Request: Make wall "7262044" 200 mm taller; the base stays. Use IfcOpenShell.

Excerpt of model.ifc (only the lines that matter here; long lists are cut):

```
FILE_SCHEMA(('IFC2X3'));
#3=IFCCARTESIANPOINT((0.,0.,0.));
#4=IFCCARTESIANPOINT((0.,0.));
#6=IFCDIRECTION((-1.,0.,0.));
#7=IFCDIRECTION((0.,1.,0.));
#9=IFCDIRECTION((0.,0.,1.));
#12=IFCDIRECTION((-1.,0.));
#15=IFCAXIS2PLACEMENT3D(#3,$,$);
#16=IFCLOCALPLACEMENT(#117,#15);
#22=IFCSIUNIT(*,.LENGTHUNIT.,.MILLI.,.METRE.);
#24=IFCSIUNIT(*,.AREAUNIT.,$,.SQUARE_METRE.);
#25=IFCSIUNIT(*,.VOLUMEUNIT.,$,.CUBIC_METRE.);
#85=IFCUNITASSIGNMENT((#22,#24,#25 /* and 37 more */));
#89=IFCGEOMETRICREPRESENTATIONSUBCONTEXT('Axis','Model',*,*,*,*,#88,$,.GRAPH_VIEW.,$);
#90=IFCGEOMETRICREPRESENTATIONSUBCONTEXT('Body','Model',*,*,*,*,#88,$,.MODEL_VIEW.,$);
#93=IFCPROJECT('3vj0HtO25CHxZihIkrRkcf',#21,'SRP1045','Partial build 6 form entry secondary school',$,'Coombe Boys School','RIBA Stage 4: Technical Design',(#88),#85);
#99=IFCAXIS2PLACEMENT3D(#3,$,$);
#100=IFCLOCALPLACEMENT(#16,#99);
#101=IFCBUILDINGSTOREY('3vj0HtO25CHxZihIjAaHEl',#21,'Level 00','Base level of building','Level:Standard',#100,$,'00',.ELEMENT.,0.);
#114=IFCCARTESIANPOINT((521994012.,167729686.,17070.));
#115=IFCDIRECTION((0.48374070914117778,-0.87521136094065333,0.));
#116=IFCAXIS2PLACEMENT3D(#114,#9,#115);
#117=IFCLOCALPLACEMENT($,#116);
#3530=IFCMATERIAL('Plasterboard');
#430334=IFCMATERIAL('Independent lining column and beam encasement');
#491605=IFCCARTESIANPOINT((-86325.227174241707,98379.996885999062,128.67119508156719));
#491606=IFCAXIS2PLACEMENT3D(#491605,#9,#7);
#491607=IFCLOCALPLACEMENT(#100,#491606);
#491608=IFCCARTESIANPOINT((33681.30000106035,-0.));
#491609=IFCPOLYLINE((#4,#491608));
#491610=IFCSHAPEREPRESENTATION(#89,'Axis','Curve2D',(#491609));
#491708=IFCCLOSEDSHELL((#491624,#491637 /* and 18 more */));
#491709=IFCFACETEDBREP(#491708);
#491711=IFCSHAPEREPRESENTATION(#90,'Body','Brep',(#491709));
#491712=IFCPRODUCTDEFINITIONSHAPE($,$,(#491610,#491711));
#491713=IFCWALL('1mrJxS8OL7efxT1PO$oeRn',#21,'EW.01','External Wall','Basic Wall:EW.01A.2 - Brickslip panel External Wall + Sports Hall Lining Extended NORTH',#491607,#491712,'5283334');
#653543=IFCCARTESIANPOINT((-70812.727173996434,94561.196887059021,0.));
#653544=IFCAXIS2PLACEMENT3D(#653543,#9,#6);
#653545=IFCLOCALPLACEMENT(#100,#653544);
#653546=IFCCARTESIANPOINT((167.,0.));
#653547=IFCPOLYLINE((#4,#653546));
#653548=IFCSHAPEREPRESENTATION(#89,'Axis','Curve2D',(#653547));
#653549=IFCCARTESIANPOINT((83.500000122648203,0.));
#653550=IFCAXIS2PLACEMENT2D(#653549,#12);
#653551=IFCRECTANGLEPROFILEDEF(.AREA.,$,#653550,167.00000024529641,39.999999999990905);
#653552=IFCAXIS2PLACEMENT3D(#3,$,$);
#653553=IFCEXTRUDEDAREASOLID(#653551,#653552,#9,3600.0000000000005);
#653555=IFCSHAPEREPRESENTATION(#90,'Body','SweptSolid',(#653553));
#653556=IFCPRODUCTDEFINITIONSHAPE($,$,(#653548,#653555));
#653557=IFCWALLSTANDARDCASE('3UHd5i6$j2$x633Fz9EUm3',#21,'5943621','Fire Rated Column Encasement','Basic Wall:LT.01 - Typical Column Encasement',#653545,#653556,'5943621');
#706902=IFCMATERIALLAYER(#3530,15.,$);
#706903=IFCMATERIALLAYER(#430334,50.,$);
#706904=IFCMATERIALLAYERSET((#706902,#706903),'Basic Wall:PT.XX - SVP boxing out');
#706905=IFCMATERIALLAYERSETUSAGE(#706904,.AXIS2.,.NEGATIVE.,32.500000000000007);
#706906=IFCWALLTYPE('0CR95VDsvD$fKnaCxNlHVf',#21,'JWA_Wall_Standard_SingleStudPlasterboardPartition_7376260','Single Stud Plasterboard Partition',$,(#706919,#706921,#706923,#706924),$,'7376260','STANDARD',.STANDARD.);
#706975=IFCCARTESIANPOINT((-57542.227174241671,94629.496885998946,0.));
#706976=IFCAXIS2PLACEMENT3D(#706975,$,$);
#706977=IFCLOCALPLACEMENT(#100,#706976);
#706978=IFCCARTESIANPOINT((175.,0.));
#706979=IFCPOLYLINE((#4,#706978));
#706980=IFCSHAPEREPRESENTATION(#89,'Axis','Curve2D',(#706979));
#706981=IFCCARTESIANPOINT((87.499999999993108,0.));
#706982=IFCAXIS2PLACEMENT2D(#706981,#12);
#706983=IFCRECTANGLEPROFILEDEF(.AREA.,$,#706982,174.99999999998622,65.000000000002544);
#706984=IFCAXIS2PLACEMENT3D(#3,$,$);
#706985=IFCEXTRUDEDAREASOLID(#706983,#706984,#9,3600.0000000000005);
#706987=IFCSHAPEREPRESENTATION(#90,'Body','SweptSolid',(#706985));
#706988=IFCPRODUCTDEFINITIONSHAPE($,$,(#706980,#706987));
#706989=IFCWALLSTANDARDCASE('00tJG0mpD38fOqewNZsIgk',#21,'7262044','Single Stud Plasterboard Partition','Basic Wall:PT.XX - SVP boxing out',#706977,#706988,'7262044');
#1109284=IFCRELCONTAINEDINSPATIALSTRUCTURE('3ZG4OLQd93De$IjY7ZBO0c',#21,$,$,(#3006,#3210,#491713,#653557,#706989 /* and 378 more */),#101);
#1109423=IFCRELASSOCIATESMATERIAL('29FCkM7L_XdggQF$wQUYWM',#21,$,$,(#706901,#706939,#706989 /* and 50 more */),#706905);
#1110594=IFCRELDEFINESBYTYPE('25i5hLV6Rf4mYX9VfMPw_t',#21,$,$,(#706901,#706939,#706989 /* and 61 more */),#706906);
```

```python
import ifcopenshell
import ifcopenshell.geom
import ifcopenshell.util.representation
import ifcopenshell.util.shape
import ifcopenshell.util.unit

model = ifcopenshell.open("model.ifc")
unit_scale = ifcopenshell.util.unit.calculate_unit_scale(model)
settings = ifcopenshell.geom.settings()


def volume(element):
    """Net volume in cubic metres, openings subtracted."""
    shape = ifcopenshell.geom.create_shape(settings, element)
    return ifcopenshell.util.shape.get_volume(shape.geometry)


wall = model.by_guid("00tJG0mpD38fOqewNZsIgk")
before = volume(wall)

body = ifcopenshell.util.representation.get_representation(wall, "Model", "Body")
solid = body.Items[0]
old_height = solid.Depth
solid.Depth += 0.2 / unit_scale
after = volume(wall)

print(f"height {old_height:g} -> {solid.Depth:g}, volume {before:.3f} -> {after:.3f} m3")

model.write("model_updated.ifc")
```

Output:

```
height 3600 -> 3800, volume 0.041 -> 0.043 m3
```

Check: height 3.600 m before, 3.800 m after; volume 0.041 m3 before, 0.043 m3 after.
